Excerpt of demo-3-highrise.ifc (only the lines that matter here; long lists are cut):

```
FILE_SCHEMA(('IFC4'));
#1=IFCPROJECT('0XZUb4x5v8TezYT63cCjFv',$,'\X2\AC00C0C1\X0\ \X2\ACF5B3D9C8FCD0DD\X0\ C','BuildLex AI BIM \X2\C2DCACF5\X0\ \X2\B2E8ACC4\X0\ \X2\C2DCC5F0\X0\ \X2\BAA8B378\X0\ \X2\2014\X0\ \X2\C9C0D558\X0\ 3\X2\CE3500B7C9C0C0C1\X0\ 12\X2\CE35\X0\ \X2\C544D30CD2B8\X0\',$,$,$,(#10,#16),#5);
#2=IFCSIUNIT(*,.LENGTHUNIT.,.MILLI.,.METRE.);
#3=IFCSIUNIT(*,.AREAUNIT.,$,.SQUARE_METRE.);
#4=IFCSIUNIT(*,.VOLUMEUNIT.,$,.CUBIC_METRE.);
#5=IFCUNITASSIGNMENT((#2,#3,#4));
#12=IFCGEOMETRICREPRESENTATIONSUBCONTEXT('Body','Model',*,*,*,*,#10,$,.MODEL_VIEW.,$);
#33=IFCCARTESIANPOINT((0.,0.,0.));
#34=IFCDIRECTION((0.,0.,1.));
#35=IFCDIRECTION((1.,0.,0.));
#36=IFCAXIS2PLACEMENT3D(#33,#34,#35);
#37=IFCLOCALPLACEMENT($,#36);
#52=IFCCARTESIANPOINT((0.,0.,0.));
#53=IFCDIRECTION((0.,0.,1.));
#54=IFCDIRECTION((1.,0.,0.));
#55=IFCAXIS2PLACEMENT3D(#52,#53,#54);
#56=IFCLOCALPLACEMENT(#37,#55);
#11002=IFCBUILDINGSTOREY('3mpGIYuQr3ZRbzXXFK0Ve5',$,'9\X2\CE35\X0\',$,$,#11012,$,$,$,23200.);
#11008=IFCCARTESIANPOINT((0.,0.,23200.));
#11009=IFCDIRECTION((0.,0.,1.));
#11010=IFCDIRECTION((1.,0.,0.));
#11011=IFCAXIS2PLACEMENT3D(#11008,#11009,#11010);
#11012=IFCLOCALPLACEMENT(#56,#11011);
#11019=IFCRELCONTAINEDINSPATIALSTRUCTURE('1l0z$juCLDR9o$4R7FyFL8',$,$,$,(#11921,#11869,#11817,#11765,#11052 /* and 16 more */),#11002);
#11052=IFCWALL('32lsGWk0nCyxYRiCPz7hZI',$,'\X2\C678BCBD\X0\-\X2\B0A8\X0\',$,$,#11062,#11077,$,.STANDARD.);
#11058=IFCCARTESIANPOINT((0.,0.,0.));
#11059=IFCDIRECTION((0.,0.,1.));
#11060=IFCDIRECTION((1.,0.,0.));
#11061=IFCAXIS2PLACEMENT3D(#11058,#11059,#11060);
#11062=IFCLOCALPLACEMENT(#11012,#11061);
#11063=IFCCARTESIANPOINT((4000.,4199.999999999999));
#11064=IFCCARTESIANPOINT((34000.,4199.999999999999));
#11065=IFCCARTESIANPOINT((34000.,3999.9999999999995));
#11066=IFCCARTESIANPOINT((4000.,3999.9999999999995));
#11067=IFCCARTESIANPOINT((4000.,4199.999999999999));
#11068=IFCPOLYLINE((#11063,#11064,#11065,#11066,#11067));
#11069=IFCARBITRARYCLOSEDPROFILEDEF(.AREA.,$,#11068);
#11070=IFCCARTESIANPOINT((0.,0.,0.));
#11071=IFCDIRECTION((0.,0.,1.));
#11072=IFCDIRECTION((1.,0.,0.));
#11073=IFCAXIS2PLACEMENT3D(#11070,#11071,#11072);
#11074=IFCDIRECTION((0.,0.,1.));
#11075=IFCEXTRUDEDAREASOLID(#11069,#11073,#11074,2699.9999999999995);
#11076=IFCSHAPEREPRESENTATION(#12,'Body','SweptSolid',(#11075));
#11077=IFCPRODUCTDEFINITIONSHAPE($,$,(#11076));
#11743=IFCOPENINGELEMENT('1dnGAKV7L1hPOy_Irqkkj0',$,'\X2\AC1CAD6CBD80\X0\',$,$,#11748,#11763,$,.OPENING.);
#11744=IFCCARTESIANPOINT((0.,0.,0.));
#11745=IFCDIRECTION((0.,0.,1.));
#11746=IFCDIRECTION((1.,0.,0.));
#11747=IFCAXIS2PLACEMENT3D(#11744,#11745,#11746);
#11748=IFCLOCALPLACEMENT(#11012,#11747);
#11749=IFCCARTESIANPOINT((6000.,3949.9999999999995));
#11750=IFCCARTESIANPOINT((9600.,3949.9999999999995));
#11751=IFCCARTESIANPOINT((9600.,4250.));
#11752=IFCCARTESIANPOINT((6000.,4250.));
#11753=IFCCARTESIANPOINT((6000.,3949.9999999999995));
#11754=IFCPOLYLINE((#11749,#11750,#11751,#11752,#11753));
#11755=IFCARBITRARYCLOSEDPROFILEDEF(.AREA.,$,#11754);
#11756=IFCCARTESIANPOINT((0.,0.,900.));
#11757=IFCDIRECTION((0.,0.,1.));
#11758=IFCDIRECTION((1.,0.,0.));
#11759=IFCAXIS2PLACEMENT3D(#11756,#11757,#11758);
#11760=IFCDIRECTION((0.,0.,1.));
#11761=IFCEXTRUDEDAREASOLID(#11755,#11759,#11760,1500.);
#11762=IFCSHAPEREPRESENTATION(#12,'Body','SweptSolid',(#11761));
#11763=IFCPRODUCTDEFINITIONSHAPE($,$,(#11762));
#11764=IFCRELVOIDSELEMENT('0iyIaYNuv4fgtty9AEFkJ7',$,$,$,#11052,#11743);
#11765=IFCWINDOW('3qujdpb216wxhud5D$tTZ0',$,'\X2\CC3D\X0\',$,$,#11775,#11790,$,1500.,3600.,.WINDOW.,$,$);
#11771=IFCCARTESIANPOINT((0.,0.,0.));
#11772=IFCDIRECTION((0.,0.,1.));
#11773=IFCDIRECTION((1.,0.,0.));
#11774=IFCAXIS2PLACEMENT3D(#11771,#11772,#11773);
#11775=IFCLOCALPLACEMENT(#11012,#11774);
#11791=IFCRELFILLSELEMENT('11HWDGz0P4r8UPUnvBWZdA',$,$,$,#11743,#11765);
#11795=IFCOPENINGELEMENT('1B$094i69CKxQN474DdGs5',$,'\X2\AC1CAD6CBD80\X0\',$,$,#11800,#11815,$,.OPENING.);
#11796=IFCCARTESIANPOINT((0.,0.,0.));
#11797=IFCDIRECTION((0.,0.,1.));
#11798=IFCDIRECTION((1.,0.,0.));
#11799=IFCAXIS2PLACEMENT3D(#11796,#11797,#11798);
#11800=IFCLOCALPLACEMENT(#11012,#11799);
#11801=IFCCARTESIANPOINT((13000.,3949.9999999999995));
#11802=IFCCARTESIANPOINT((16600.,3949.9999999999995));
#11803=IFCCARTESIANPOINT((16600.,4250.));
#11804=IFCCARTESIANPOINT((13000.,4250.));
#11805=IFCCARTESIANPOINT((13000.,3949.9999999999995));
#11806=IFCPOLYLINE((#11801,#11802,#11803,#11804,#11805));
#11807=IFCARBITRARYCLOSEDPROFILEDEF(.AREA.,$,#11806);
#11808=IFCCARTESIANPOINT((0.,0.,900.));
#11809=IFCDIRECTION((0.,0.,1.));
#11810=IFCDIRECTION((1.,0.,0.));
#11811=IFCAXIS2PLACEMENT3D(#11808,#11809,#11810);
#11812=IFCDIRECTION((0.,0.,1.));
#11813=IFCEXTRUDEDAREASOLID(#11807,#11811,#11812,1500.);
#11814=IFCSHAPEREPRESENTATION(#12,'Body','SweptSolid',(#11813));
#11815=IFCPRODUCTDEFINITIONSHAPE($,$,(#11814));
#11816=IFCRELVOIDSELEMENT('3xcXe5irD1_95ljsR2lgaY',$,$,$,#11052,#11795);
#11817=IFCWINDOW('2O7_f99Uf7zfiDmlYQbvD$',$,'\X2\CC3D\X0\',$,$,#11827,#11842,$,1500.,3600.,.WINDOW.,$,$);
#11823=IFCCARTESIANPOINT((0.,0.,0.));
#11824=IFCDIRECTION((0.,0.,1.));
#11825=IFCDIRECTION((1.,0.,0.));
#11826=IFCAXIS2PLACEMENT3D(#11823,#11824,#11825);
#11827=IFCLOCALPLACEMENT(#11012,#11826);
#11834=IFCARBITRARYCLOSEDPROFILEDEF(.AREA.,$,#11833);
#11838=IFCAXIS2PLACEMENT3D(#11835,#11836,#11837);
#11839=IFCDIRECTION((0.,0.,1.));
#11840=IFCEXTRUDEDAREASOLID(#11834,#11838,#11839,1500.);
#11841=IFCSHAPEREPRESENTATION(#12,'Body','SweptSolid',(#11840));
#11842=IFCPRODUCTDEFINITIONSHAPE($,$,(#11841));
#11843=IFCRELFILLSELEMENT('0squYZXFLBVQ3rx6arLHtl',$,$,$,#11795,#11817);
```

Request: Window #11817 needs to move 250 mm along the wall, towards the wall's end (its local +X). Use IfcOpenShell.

```python
import ifcopenshell
import ifcopenshell.api.geometry
import ifcopenshell.util.placement
import ifcopenshell.util.unit

model = ifcopenshell.open("demo-3-highrise.ifc")
unit_scale = ifcopenshell.util.unit.calculate_unit_scale(model)

window = model.by_id(11817)
opening = window.FillsVoids[0].RelatingOpeningElement
wall = opening.VoidsElements[0].RelatingBuildingElement

wall_matrix = ifcopenshell.util.placement.get_local_placement(wall.ObjectPlacement)
shift = wall_matrix[:3, 0] * 0.25 / unit_scale
before = ifcopenshell.util.placement.get_local_placement(window.ObjectPlacement)[:3, 3].copy()

# The window is not placed relative to its opening, so move both.
for product in (opening, window):
    matrix = ifcopenshell.util.placement.get_local_placement(product.ObjectPlacement)
    matrix[:3, 3] += shift
    ifcopenshell.api.geometry.edit_object_placement(model, product=product, matrix=matrix, is_si=False)

after = ifcopenshell.util.placement.get_local_placement(window.ObjectPlacement)[:3, 3]
print("window moved by", (after - before).round(3) + 0.0)

model.write("demo-3-highrise_updated.ifc")
```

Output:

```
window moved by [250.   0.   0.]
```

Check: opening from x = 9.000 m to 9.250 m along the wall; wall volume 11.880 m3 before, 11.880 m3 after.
